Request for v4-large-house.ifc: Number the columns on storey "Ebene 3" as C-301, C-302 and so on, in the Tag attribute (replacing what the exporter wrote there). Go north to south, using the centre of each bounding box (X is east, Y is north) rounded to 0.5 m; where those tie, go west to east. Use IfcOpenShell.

First a look at what the model holds.

```python
import ifcopenshell
import ifcopenshell.util.element
import ifcopenshell.util.placement

model = ifcopenshell.open("v4-large-house.ifc")
print(model.schema)
storey = next(s for s in model.by_type("IfcBuildingStorey") if s.Name == "Ebene 3")
columns = [e for e in ifcopenshell.util.element.get_decomposition(storey) if e.is_a("IfcColumn")]
for e in sorted(columns, key=lambda e: e.id()):
    origin = ifcopenshell.util.placement.get_local_placement(e.ObjectPlacement)[:3, 3]
    print(e.id(), e.Tag, e.Name, origin.round(2) + 0.0, sep=" | ")
```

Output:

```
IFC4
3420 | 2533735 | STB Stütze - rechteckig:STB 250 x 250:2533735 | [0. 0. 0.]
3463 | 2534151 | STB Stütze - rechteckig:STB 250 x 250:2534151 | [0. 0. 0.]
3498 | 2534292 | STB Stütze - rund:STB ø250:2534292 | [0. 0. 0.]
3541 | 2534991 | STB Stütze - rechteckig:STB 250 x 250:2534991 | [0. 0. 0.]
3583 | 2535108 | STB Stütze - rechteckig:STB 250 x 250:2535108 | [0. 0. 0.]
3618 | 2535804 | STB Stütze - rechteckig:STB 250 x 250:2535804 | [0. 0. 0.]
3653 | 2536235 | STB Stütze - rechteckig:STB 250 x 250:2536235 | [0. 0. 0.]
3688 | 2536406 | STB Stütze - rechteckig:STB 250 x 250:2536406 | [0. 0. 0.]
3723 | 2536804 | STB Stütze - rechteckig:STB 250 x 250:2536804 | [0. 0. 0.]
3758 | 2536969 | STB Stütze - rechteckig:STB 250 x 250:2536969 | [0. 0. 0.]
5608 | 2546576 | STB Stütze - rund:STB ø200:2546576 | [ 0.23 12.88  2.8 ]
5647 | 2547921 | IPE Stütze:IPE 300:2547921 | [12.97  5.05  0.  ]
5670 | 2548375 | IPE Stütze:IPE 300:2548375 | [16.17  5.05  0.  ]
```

```python
import ifcopenshell
import ifcopenshell.geom
import ifcopenshell.util.element
import ifcopenshell.util.shape

model = ifcopenshell.open("v4-large-house.ifc")
settings = ifcopenshell.geom.settings()
settings.set("use-world-coords", True)


def centre(element):
    shape = ifcopenshell.geom.create_shape(settings, element)
    return ifcopenshell.util.shape.get_bbox_centroid(shape.geometry)


storey = next(s for s in model.by_type("IfcBuildingStorey") if s.Name == "Ebene 3")
columns = [e for e in ifcopenshell.util.element.get_decomposition(storey) if e.is_a("IfcColumn")]

# Insertion points can sit at a corner or the storey origin, so sort by the geometry (in metres).
centres = {e: centre(e) for e in columns}
columns.sort(key=lambda e: (-round(centres[e][1] / 0.5), centres[e][0]))

for i, e in enumerate(columns, start=1):
    number = f"C-3{i:02d}"
    e.Tag = number
    print(e.id(), number)

model.write("v4-large-house-out.ifc")
```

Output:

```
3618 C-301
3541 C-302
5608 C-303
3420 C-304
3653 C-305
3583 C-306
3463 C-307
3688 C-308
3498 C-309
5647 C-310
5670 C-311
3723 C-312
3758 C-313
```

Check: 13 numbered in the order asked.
